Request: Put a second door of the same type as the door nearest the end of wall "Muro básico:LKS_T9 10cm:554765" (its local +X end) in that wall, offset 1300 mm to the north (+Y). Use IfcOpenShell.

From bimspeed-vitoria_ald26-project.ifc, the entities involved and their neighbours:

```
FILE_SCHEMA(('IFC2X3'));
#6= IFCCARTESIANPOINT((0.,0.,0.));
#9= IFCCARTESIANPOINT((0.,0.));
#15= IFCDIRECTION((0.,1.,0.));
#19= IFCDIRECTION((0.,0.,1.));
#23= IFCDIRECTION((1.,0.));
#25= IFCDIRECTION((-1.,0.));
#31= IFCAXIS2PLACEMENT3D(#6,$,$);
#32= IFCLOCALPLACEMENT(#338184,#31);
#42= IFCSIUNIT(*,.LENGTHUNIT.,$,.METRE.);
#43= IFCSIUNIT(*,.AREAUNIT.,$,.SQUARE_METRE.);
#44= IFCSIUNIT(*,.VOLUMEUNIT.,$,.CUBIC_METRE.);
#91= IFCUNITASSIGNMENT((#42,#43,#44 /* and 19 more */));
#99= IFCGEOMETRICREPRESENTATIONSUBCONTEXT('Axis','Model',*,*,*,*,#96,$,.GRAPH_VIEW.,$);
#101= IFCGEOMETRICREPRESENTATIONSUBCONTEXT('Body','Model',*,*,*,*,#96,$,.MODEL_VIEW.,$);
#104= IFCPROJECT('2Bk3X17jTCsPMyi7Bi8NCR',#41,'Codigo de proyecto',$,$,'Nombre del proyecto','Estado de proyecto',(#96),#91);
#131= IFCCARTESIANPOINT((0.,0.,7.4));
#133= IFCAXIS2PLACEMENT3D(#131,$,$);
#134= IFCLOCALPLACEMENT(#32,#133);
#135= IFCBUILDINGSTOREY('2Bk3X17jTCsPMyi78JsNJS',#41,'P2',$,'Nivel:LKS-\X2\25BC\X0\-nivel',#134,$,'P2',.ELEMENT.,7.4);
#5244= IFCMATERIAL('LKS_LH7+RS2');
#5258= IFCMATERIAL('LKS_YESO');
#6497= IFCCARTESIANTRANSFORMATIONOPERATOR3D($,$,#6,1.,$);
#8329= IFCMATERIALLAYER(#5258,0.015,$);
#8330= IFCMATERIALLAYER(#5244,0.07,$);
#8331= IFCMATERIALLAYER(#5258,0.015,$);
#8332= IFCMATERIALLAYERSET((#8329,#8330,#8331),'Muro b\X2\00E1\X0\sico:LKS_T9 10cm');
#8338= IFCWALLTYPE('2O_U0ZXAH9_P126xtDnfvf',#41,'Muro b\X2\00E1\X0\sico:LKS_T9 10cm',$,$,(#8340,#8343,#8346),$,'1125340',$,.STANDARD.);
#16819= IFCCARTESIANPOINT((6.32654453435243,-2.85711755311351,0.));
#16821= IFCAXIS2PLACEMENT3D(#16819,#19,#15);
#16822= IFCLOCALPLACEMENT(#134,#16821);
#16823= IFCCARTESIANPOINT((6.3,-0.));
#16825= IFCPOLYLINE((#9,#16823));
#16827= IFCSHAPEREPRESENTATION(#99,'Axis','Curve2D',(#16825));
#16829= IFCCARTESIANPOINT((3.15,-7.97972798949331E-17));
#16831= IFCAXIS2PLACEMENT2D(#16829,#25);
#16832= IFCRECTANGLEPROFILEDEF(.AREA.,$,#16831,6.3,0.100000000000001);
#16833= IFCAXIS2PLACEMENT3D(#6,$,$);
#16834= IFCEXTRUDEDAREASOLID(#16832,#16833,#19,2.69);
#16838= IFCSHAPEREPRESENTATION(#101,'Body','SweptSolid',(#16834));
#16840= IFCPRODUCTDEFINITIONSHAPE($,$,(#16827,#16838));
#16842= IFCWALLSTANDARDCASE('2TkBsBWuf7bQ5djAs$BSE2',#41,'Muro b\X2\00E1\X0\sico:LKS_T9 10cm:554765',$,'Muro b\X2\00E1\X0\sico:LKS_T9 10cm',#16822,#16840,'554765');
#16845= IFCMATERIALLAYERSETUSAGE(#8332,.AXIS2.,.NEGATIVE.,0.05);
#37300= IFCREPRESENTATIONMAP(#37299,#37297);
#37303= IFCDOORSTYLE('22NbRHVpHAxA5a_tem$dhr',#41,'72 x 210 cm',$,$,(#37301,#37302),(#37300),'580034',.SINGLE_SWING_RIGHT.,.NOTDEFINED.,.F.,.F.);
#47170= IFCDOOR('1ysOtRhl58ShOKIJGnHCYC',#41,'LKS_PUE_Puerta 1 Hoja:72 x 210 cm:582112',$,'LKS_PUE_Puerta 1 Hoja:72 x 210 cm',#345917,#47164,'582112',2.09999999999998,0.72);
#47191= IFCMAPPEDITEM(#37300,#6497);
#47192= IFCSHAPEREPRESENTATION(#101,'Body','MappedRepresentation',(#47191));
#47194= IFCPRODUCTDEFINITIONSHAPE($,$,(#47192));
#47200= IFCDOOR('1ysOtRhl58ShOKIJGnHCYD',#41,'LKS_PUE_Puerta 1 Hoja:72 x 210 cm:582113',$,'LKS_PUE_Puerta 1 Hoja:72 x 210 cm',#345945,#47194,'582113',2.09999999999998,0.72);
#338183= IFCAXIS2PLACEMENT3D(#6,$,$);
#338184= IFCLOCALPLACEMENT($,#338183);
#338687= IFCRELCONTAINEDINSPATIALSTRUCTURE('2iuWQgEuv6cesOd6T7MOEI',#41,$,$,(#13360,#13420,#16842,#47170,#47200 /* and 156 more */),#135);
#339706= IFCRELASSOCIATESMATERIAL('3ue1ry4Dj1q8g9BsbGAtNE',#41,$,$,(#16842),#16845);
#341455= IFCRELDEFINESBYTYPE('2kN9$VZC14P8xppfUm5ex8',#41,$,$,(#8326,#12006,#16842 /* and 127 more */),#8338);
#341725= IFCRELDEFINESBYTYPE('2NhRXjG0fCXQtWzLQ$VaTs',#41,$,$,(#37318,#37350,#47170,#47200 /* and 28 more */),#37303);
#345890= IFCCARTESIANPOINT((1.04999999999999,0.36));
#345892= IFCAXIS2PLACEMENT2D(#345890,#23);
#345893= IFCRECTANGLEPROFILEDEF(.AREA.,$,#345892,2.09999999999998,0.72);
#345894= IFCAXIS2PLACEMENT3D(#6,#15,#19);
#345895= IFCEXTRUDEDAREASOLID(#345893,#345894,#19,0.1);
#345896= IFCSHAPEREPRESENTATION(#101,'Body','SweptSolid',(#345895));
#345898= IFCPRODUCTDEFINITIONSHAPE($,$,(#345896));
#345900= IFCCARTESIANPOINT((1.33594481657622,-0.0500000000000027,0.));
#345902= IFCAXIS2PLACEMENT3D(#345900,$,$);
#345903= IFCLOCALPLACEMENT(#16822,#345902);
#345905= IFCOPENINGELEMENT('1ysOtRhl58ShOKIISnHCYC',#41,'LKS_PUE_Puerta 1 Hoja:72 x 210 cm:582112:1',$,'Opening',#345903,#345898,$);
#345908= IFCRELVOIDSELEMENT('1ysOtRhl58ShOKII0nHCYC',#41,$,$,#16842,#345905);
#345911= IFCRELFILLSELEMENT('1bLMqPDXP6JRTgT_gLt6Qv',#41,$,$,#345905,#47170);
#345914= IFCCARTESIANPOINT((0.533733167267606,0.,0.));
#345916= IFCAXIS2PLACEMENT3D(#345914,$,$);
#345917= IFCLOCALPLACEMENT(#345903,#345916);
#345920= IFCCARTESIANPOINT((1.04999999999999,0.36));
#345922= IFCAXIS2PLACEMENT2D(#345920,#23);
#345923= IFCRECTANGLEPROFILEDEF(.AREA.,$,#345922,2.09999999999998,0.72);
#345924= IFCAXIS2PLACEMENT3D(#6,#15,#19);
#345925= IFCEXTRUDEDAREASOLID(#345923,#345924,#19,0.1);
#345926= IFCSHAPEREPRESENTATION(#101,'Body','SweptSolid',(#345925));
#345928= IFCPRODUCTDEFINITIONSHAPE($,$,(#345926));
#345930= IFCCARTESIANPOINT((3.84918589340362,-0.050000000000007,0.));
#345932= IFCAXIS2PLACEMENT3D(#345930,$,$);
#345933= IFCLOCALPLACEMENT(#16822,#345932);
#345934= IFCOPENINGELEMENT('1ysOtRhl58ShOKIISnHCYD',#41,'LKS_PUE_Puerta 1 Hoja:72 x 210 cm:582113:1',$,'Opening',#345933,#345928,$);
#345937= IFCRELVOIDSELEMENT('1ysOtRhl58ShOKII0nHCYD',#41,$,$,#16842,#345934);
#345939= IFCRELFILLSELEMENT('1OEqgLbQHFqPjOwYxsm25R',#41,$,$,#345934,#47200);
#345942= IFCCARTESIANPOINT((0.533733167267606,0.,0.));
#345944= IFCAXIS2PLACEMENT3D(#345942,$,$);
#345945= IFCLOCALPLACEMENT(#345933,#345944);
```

```python
import ifcopenshell
import ifcopenshell.api.feature
import ifcopenshell.api.geometry
import ifcopenshell.api.root
import ifcopenshell.geom
import ifcopenshell.util.element
import ifcopenshell.util.placement
import ifcopenshell.util.shape

model = ifcopenshell.open("bimspeed-vitoria_ald26-project.ifc")
settings = ifcopenshell.geom.settings()


def volume(element):
    """Net volume in cubic metres, openings subtracted."""
    shape = ifcopenshell.geom.create_shape(settings, element)
    return ifcopenshell.util.shape.get_volume(shape.geometry)


def reuse_history(source, copy):
    """copy_class also copies each property set's owner history, people and application; keep the originals."""
    for rel in copy.IsDefinedBy:
        if rel.is_a("IfcRelDefinesByProperties") and (history := rel.RelatingPropertyDefinition.OwnerHistory):
            rel.RelatingPropertyDefinition.OwnerHistory = source.OwnerHistory
            ifcopenshell.util.element.remove_deep2(model, history)


door = model.by_id(47200)
opening = door.FillsVoids[0].RelatingOpeningElement
wall = opening.VoidsElements[0].RelatingBuildingElement
before = volume(wall)
shift = ifcopenshell.util.placement.get_local_placement(wall.ObjectPlacement)[:3, 0] * 1.3

# copy_class copies the void relationship, type, container and properties, but no geometry.
new_opening = ifcopenshell.api.root.copy_class(model, product=opening)
new_opening.Representation = ifcopenshell.util.element.copy_deep(
    model, opening.Representation, exclude=["IfcGeometricRepresentationContext", "IfcRepresentationMap"]
)
new_opening.Name = "LKS_PUE_Puerta 1 Hoja:72 x 210 cm"
new_door = ifcopenshell.api.root.copy_class(model, product=door)
new_door.Representation = ifcopenshell.util.element.copy_deep(
    model, door.Representation, exclude=["IfcGeometricRepresentationContext", "IfcRepresentationMap"]
)
new_door.Name = "LKS_PUE_Puerta 1 Hoja:72 x 210 cm"
new_door.Tag = None
reuse_history(door, new_door)
fills = ifcopenshell.api.feature.add_filling(model, opening=new_opening, element=new_door)
fills.OwnerHistory = new_door.OwnerHistory  # required in IFC2X3

for old, new in ((opening, new_opening), (door, new_door)):
    matrix = ifcopenshell.util.placement.get_local_placement(old.ObjectPlacement)
    matrix[:3, 3] += shift
    ifcopenshell.api.geometry.edit_object_placement(model, product=new, matrix=matrix, is_si=False)

after = volume(wall)

print(f"wall volume {before:.3f} -> {after:.3f} m3")

model.write("bimspeed-vitoria_ald26-project_edited.ifc")
```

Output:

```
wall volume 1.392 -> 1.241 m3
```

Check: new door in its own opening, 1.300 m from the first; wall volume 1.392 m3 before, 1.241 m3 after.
